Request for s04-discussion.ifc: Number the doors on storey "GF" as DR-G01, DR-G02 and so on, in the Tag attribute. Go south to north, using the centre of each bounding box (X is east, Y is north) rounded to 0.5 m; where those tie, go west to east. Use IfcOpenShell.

First a look at what the model holds.

```python
import ifcopenshell
import ifcopenshell.util.element
import ifcopenshell.util.placement

model = ifcopenshell.open("s04-discussion.ifc")
print(model.schema)
storey = next(s for s in model.by_type("IfcBuildingStorey") if s.Name == "GF")
doors = [e for e in ifcopenshell.util.element.get_decomposition(storey) if e.is_a("IfcDoor")]
for e in sorted(doors, key=lambda e: e.id()):
    origin = ifcopenshell.util.placement.get_local_placement(e.ObjectPlacement)[:3, 3]
    print(e.id(), e.Tag, e.Name, origin.round(2) + 0.0, sep=" | ")
```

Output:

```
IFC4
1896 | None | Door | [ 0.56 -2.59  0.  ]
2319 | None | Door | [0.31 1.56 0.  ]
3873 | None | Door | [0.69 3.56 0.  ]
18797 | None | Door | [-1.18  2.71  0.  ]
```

```python
import ifcopenshell
import ifcopenshell.geom
import ifcopenshell.util.element
import ifcopenshell.util.shape

model = ifcopenshell.open("s04-discussion.ifc")
settings = ifcopenshell.geom.settings()
settings.set("use-world-coords", True)


def centre(element):
    shape = ifcopenshell.geom.create_shape(settings, element)
    return ifcopenshell.util.shape.get_bbox_centroid(shape.geometry)


storey = next(s for s in model.by_type("IfcBuildingStorey") if s.Name == "GF")
doors = [e for e in ifcopenshell.util.element.get_decomposition(storey) if e.is_a("IfcDoor")]

# Insertion points can sit at a corner or the storey origin, so sort by the geometry (in metres).
centres = {e: centre(e) for e in doors}
doors.sort(key=lambda e: (round(centres[e][1] / 0.5), centres[e][0]))

for i, e in enumerate(doors, start=1):
    number = f"DR-G{i:02d}"
    e.Tag = number
    print(e.id(), number)

model.write("s04-discussion_v2.ifc")
```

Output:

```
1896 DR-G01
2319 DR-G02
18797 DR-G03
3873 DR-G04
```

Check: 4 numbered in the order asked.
